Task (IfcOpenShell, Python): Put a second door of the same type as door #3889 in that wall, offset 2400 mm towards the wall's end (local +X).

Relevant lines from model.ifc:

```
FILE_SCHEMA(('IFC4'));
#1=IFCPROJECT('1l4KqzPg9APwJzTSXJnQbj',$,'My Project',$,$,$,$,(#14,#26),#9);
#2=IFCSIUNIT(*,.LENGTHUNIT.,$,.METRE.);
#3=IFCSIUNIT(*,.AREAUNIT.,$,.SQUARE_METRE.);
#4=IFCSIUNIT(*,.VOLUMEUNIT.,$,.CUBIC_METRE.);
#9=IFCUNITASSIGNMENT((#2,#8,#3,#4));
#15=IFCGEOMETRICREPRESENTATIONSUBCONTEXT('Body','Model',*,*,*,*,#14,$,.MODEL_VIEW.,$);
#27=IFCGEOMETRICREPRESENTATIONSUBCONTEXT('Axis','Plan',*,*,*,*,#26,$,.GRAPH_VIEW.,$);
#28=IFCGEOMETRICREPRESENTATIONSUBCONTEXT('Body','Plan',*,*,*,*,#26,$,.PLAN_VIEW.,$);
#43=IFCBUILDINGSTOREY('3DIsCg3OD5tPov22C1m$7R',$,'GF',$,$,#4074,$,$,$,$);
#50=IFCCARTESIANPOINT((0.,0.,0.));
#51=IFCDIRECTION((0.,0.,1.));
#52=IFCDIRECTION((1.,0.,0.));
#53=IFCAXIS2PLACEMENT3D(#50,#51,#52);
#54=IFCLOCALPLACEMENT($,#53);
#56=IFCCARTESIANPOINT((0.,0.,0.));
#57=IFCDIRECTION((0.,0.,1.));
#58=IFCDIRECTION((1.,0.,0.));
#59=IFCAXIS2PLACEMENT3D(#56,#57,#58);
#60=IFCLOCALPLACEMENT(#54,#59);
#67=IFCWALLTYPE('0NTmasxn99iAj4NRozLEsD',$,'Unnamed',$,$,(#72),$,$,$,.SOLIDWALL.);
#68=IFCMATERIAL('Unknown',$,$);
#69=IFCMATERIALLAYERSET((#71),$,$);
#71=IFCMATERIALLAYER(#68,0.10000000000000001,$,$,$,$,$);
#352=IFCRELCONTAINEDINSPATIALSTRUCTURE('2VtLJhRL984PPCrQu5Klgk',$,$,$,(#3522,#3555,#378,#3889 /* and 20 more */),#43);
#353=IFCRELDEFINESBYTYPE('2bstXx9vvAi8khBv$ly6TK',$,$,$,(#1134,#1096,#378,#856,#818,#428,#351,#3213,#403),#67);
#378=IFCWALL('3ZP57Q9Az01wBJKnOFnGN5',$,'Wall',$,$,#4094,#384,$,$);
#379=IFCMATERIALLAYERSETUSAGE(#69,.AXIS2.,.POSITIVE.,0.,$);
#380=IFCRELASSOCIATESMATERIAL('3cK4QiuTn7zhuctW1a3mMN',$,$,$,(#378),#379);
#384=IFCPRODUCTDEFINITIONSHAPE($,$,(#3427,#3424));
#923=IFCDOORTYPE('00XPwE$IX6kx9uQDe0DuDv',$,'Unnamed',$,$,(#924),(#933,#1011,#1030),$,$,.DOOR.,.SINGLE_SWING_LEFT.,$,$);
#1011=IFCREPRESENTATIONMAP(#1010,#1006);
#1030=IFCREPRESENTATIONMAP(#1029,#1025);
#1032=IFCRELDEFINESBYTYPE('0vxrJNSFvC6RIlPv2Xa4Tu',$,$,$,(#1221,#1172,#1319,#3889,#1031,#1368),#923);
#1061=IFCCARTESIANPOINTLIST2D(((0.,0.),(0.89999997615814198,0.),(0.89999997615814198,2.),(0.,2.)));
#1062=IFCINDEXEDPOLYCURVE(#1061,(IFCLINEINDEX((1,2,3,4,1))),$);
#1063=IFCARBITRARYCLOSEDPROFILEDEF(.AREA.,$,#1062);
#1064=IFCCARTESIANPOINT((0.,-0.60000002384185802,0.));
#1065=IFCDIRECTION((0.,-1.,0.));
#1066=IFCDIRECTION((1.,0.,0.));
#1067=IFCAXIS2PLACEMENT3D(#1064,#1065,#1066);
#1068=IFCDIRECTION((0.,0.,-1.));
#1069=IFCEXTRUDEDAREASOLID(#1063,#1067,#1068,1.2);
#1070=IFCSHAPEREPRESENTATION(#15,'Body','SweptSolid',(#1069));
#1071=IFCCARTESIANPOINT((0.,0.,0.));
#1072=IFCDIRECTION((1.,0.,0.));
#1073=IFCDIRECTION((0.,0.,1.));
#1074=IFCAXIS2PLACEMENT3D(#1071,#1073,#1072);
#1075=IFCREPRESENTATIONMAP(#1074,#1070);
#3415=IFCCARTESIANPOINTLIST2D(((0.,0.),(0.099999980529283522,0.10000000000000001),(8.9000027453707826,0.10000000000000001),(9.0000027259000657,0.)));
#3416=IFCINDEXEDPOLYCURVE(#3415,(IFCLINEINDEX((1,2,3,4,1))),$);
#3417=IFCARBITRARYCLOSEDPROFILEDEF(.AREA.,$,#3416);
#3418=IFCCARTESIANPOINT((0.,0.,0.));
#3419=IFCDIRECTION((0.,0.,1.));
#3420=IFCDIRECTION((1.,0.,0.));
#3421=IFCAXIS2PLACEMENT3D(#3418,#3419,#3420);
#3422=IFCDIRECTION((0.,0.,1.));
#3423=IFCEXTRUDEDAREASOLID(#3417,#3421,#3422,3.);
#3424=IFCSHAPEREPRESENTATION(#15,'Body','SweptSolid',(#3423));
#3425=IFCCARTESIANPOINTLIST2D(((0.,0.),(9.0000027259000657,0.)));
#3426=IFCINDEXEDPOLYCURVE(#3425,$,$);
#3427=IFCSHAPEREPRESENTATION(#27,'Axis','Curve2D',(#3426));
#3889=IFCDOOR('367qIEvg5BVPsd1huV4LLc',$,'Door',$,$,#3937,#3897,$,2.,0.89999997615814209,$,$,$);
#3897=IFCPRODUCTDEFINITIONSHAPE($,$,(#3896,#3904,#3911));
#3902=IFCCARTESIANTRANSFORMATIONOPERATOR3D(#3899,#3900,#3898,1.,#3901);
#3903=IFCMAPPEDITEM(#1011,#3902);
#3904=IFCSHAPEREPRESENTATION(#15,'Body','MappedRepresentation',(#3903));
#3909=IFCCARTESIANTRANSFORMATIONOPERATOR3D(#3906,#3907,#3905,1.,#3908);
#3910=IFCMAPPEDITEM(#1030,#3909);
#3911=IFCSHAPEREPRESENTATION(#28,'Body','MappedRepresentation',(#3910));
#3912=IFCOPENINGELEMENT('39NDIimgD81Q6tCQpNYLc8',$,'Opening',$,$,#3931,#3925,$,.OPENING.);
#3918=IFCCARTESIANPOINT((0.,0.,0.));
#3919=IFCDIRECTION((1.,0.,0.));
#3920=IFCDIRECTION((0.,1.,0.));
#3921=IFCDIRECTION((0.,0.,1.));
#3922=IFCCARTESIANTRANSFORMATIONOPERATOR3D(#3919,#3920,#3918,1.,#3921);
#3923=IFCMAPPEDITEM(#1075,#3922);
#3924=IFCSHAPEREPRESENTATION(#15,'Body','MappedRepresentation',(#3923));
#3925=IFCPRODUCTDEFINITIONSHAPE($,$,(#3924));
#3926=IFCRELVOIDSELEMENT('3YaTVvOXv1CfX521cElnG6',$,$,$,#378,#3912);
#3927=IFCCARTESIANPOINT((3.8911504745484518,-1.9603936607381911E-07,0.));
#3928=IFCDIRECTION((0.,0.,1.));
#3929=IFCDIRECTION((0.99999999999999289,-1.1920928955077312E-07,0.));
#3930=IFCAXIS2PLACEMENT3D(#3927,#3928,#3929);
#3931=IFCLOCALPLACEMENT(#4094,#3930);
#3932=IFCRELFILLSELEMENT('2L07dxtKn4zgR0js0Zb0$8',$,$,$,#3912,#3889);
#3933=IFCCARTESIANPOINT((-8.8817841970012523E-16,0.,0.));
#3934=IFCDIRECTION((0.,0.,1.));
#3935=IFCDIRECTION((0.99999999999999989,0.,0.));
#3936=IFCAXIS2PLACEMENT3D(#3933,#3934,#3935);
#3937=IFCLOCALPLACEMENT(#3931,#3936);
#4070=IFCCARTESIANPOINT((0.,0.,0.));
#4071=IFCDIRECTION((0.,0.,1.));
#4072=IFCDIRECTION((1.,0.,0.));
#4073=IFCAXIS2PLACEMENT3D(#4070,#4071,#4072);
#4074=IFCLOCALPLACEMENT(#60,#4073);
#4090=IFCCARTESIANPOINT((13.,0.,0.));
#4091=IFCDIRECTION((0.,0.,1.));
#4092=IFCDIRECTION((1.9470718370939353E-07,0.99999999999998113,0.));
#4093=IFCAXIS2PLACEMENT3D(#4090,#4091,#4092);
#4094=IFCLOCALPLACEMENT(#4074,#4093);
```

```python
import ifcopenshell
import ifcopenshell.api.feature
import ifcopenshell.api.geometry
import ifcopenshell.api.root
import ifcopenshell.geom
import ifcopenshell.util.element
import ifcopenshell.util.placement
import ifcopenshell.util.shape
import ifcopenshell.util.unit

model = ifcopenshell.open("model.ifc")
unit_scale = ifcopenshell.util.unit.calculate_unit_scale(model)
settings = ifcopenshell.geom.settings()


def volume(element):
    """Net volume in cubic metres, openings subtracted."""
    shape = ifcopenshell.geom.create_shape(settings, element)
    return ifcopenshell.util.shape.get_volume(shape.geometry)


door = model.by_guid("367qIEvg5BVPsd1huV4LLc")
opening = door.FillsVoids[0].RelatingOpeningElement
wall = opening.VoidsElements[0].RelatingBuildingElement
before = volume(wall)
shift = ifcopenshell.util.placement.get_local_placement(wall.ObjectPlacement)[:3, 0] * 2.4 / unit_scale

# copy_class copies the void relationship, type, container and properties, but no geometry.
new_opening = ifcopenshell.api.root.copy_class(model, product=opening)
new_opening.Representation = ifcopenshell.util.element.copy_deep(
    model, opening.Representation, exclude=["IfcGeometricRepresentationContext", "IfcRepresentationMap"]
)
new_door = ifcopenshell.api.root.copy_class(model, product=door)
new_door.Representation = ifcopenshell.util.element.copy_deep(
    model, door.Representation, exclude=["IfcGeometricRepresentationContext", "IfcRepresentationMap"]
)
ifcopenshell.api.feature.add_filling(model, opening=new_opening, element=new_door)

for old, new in ((opening, new_opening), (door, new_door)):
    matrix = ifcopenshell.util.placement.get_local_placement(old.ObjectPlacement)
    matrix[:3, 3] += shift
    ifcopenshell.api.geometry.edit_object_placement(model, product=new, matrix=matrix, is_si=False)

after = volume(wall)

print(f"wall volume {before:.3f} -> {after:.3f} m3")

model.write("model_v2.ifc")
```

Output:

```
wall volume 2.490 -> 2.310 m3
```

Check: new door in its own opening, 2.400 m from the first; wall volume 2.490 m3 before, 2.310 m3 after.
